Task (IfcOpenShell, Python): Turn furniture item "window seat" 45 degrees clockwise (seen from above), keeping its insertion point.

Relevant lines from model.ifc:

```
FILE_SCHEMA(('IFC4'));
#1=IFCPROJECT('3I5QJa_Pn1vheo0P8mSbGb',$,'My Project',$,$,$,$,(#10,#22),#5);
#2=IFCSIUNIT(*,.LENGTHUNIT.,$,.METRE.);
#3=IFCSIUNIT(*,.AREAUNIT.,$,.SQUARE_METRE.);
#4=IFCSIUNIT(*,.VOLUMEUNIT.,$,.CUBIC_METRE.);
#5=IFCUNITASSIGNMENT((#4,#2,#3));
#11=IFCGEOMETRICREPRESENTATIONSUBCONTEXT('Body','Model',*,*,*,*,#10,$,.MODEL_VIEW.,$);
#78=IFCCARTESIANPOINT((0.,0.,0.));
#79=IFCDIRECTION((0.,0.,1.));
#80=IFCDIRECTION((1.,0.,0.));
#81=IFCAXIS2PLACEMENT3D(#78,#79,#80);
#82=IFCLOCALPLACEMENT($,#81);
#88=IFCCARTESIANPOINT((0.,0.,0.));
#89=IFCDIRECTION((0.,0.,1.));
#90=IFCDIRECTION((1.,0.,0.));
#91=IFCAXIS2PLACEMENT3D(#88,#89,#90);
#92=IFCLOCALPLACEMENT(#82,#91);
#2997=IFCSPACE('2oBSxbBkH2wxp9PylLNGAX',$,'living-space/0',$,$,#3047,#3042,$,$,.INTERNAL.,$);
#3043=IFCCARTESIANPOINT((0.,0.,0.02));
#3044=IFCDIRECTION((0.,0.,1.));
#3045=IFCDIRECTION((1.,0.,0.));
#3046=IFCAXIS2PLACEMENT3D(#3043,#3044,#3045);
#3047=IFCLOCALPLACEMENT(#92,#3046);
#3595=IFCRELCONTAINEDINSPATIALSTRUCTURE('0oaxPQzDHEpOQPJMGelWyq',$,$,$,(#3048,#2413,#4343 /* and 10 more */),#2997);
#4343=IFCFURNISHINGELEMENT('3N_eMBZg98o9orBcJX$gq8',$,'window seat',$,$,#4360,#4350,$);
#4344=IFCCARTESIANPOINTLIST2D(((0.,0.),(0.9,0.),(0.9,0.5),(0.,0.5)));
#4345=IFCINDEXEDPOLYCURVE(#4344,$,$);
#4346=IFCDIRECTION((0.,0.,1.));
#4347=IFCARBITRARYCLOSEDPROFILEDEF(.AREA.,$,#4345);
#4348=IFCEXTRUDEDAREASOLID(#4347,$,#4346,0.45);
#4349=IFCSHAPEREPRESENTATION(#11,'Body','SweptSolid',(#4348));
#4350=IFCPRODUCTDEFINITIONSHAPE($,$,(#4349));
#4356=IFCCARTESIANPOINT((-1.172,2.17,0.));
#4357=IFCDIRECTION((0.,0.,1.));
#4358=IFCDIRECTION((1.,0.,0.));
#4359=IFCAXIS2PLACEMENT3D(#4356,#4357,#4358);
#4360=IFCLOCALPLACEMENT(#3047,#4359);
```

```python
import ifcopenshell
import ifcopenshell.api.geometry
import ifcopenshell.util.placement

model = ifcopenshell.open("model.ifc")

item = model.by_guid("3N_eMBZg98o9orBcJX$gq8")
matrix = ifcopenshell.util.placement.get_local_placement(item.ObjectPlacement)
matrix = matrix @ ifcopenshell.util.placement.rotation(-45, "Z")
ifcopenshell.api.geometry.edit_object_placement(model, product=item, matrix=matrix, is_si=False)

print(ifcopenshell.util.placement.get_local_placement(item.ObjectPlacement).round(3) + 0.0)

model.write("model-out.ifc")
```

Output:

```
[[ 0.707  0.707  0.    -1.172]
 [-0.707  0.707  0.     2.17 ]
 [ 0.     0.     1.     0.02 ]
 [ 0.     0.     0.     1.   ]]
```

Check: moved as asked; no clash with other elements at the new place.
